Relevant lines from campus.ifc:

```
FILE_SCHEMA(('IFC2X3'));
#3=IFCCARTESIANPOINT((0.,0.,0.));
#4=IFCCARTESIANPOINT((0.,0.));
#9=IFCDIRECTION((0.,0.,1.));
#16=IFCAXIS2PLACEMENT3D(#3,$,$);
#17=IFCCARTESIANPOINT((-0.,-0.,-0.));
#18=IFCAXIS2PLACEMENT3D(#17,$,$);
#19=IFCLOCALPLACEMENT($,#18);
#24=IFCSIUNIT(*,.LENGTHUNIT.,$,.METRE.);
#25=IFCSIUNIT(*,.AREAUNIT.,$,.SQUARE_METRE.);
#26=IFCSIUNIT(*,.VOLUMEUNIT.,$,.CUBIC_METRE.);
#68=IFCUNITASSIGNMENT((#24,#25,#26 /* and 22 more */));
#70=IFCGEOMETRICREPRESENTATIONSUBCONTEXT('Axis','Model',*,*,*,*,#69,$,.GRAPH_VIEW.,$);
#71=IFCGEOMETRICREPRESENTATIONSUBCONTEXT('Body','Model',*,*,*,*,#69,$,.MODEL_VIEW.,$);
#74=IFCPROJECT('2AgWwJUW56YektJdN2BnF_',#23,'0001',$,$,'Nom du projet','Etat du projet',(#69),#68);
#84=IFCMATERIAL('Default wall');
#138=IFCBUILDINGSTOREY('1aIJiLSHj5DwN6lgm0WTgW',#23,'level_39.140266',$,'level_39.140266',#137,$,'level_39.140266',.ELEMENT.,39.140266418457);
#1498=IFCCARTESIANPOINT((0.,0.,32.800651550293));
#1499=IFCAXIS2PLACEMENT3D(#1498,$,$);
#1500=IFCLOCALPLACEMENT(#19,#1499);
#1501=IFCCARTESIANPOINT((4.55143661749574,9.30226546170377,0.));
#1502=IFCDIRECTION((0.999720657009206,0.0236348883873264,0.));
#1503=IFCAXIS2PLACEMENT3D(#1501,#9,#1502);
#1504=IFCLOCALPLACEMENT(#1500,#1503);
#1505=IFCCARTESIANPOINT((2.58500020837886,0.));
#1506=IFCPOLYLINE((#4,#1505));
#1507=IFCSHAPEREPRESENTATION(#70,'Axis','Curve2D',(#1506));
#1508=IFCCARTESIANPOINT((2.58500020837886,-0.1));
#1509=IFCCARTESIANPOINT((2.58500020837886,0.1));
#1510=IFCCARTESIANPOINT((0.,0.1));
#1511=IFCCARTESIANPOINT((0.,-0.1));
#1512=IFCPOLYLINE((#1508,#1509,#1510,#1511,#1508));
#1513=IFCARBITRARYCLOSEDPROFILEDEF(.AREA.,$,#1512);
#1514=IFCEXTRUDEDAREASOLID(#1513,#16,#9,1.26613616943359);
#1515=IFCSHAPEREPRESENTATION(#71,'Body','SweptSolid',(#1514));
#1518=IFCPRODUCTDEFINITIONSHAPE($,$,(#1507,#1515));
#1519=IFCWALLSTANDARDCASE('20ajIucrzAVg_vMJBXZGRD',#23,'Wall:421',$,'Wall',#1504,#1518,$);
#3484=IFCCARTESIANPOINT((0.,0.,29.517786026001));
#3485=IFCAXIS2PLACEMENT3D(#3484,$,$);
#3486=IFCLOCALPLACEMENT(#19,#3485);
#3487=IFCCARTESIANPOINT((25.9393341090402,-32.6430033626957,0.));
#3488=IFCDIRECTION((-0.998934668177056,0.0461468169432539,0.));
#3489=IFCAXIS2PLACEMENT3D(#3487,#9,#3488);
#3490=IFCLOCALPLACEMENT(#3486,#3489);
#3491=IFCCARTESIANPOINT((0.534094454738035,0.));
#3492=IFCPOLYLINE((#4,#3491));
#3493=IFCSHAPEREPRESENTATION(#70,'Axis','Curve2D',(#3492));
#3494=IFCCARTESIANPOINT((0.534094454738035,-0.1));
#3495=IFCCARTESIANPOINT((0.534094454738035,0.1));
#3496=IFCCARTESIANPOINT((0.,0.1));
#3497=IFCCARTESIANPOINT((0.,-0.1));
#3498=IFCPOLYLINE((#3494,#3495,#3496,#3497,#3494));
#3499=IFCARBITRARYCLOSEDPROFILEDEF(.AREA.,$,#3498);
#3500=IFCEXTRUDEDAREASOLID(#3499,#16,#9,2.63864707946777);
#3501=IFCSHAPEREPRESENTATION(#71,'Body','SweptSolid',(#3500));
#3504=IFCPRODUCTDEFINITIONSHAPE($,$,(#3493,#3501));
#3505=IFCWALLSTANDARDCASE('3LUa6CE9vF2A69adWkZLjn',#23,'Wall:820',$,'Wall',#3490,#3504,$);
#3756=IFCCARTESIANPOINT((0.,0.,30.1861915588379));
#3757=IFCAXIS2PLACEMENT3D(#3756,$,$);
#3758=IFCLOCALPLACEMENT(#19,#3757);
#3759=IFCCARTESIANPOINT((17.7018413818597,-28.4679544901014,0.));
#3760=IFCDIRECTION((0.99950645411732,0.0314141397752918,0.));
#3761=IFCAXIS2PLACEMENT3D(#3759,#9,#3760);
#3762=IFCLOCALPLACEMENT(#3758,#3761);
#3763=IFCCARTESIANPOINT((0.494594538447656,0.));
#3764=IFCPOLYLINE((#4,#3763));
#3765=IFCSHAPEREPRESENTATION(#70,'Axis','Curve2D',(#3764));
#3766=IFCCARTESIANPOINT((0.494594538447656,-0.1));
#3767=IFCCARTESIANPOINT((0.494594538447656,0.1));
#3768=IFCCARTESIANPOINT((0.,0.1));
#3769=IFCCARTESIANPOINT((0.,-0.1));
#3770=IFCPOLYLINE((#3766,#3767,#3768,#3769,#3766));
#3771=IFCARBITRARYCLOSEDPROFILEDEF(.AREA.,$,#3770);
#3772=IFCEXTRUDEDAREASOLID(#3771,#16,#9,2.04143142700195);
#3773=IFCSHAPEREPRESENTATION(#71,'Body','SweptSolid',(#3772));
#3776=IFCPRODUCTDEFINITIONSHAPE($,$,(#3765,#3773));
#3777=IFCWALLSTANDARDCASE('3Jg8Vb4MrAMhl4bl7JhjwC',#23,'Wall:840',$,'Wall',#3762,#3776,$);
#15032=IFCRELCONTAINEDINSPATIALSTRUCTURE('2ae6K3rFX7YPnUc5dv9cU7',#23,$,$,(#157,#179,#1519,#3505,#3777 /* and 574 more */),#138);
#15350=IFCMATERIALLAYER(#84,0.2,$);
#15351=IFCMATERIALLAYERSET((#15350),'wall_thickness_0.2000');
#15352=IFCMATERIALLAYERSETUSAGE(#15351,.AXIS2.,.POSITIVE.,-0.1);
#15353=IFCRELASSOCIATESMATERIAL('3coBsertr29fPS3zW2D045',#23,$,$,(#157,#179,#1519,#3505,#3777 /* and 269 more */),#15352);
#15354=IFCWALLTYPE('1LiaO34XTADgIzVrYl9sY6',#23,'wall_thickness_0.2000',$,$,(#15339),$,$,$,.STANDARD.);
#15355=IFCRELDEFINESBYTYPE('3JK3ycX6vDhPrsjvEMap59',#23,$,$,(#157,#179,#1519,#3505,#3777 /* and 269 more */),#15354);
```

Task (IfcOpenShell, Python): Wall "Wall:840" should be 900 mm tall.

```python
import ifcopenshell
import ifcopenshell.geom
import ifcopenshell.util.representation
import ifcopenshell.util.shape
import ifcopenshell.util.unit

model = ifcopenshell.open("campus.ifc")
unit_scale = ifcopenshell.util.unit.calculate_unit_scale(model)
settings = ifcopenshell.geom.settings()


def volume(element):
    """Net volume in cubic metres, openings subtracted."""
    shape = ifcopenshell.geom.create_shape(settings, element)
    return ifcopenshell.util.shape.get_volume(shape.geometry)


wall = model.by_guid("3Jg8Vb4MrAMhl4bl7JhjwC")
before = volume(wall)

body = ifcopenshell.util.representation.get_representation(wall, "Model", "Body")
solid = body.Items[0]
old_height = solid.Depth
solid.Depth = 0.9 / unit_scale
after = volume(wall)

print(f"height {old_height:g} -> {solid.Depth:g}, volume {before:.3f} -> {after:.3f} m3")

model.write("campus-out.ifc")
```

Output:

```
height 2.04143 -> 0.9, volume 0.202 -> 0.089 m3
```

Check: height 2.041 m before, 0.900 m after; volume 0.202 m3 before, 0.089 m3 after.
